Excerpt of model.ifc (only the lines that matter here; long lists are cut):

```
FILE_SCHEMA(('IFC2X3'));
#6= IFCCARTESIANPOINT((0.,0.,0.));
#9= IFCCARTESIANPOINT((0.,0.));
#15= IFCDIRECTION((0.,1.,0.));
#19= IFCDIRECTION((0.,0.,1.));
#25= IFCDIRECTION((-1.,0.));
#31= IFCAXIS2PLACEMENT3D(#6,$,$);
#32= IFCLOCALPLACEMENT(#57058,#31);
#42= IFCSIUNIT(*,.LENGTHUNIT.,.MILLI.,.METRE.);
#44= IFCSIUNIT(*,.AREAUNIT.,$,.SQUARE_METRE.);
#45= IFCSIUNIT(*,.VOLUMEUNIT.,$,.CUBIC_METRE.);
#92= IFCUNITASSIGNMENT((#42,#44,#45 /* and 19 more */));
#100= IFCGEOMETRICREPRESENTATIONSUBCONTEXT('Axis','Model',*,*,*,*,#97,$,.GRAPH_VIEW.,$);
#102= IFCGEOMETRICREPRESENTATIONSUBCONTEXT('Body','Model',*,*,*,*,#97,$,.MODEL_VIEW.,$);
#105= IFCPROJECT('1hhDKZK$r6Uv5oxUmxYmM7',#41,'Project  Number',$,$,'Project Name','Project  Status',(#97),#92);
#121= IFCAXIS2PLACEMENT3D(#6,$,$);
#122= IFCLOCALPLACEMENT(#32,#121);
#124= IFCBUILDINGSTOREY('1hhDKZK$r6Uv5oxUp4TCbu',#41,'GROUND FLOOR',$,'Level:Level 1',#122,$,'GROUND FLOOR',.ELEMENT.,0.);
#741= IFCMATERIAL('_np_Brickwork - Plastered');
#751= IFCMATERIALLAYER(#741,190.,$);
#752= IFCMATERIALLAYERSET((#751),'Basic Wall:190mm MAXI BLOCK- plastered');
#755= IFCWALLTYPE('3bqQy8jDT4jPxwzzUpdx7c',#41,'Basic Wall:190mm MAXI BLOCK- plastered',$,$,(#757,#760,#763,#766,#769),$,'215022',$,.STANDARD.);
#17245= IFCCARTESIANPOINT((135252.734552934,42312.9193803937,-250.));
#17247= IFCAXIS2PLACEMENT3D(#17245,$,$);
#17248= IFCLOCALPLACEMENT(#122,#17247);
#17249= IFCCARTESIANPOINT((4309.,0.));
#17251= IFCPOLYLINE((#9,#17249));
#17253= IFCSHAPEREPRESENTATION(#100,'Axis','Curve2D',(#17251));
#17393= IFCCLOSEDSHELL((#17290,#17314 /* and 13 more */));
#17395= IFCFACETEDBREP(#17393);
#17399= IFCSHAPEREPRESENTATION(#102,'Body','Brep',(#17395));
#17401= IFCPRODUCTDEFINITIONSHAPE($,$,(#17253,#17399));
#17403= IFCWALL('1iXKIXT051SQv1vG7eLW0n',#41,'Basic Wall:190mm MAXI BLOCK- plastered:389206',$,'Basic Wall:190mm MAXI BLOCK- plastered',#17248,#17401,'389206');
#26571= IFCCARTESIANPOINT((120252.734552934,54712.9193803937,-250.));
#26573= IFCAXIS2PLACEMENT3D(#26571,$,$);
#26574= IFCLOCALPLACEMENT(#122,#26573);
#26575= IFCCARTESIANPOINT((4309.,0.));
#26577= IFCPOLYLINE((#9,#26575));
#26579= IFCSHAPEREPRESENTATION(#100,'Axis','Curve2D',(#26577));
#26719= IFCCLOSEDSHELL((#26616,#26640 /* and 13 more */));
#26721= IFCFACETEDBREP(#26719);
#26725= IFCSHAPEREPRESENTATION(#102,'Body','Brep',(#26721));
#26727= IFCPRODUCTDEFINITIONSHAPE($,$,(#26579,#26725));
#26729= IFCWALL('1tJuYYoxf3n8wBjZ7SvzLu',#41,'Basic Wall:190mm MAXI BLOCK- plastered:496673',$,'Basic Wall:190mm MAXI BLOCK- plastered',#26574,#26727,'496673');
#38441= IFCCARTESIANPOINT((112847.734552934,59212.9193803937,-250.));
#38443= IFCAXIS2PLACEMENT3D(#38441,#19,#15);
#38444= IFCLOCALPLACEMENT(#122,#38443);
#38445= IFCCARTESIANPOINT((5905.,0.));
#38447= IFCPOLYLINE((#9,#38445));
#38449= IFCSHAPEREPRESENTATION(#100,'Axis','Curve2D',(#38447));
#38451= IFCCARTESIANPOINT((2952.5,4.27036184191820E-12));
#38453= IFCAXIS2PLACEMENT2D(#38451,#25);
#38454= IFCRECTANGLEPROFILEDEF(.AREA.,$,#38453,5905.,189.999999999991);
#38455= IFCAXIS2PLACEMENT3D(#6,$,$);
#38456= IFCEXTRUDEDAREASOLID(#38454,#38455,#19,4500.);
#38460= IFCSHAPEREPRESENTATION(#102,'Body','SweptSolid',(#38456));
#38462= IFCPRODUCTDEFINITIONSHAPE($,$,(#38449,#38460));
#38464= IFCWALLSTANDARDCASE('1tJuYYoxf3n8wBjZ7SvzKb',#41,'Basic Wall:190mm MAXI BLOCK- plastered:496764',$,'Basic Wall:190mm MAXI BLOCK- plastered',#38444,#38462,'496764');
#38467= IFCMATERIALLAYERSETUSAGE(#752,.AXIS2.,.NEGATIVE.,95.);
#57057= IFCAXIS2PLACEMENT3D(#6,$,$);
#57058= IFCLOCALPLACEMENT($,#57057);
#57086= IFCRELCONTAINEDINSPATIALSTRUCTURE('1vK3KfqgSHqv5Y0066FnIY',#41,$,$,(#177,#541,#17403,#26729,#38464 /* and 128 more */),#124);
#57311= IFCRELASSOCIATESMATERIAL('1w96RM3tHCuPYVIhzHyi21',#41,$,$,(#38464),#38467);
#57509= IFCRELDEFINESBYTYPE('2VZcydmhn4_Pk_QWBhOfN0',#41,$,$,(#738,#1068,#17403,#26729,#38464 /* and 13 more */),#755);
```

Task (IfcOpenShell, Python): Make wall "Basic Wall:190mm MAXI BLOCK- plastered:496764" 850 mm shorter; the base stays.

```python
import ifcopenshell
import ifcopenshell.geom
import ifcopenshell.util.representation
import ifcopenshell.util.shape
import ifcopenshell.util.unit

model = ifcopenshell.open("model.ifc")
unit_scale = ifcopenshell.util.unit.calculate_unit_scale(model)
settings = ifcopenshell.geom.settings()


def volume(element):
    """Net volume in cubic metres, openings subtracted."""
    shape = ifcopenshell.geom.create_shape(settings, element)
    return ifcopenshell.util.shape.get_volume(shape.geometry)


wall = model.by_id(38464)
before = volume(wall)

body = ifcopenshell.util.representation.get_representation(wall, "Model", "Body")
solid = body.Items[0]
old_height = solid.Depth
solid.Depth -= 0.85 / unit_scale
after = volume(wall)

print(f"height {old_height:g} -> {solid.Depth:g}, volume {before:.3f} -> {after:.3f} m3")

model.write("model_edited.ifc")
```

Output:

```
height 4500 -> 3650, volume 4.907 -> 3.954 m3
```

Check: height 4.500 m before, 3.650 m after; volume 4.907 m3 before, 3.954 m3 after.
